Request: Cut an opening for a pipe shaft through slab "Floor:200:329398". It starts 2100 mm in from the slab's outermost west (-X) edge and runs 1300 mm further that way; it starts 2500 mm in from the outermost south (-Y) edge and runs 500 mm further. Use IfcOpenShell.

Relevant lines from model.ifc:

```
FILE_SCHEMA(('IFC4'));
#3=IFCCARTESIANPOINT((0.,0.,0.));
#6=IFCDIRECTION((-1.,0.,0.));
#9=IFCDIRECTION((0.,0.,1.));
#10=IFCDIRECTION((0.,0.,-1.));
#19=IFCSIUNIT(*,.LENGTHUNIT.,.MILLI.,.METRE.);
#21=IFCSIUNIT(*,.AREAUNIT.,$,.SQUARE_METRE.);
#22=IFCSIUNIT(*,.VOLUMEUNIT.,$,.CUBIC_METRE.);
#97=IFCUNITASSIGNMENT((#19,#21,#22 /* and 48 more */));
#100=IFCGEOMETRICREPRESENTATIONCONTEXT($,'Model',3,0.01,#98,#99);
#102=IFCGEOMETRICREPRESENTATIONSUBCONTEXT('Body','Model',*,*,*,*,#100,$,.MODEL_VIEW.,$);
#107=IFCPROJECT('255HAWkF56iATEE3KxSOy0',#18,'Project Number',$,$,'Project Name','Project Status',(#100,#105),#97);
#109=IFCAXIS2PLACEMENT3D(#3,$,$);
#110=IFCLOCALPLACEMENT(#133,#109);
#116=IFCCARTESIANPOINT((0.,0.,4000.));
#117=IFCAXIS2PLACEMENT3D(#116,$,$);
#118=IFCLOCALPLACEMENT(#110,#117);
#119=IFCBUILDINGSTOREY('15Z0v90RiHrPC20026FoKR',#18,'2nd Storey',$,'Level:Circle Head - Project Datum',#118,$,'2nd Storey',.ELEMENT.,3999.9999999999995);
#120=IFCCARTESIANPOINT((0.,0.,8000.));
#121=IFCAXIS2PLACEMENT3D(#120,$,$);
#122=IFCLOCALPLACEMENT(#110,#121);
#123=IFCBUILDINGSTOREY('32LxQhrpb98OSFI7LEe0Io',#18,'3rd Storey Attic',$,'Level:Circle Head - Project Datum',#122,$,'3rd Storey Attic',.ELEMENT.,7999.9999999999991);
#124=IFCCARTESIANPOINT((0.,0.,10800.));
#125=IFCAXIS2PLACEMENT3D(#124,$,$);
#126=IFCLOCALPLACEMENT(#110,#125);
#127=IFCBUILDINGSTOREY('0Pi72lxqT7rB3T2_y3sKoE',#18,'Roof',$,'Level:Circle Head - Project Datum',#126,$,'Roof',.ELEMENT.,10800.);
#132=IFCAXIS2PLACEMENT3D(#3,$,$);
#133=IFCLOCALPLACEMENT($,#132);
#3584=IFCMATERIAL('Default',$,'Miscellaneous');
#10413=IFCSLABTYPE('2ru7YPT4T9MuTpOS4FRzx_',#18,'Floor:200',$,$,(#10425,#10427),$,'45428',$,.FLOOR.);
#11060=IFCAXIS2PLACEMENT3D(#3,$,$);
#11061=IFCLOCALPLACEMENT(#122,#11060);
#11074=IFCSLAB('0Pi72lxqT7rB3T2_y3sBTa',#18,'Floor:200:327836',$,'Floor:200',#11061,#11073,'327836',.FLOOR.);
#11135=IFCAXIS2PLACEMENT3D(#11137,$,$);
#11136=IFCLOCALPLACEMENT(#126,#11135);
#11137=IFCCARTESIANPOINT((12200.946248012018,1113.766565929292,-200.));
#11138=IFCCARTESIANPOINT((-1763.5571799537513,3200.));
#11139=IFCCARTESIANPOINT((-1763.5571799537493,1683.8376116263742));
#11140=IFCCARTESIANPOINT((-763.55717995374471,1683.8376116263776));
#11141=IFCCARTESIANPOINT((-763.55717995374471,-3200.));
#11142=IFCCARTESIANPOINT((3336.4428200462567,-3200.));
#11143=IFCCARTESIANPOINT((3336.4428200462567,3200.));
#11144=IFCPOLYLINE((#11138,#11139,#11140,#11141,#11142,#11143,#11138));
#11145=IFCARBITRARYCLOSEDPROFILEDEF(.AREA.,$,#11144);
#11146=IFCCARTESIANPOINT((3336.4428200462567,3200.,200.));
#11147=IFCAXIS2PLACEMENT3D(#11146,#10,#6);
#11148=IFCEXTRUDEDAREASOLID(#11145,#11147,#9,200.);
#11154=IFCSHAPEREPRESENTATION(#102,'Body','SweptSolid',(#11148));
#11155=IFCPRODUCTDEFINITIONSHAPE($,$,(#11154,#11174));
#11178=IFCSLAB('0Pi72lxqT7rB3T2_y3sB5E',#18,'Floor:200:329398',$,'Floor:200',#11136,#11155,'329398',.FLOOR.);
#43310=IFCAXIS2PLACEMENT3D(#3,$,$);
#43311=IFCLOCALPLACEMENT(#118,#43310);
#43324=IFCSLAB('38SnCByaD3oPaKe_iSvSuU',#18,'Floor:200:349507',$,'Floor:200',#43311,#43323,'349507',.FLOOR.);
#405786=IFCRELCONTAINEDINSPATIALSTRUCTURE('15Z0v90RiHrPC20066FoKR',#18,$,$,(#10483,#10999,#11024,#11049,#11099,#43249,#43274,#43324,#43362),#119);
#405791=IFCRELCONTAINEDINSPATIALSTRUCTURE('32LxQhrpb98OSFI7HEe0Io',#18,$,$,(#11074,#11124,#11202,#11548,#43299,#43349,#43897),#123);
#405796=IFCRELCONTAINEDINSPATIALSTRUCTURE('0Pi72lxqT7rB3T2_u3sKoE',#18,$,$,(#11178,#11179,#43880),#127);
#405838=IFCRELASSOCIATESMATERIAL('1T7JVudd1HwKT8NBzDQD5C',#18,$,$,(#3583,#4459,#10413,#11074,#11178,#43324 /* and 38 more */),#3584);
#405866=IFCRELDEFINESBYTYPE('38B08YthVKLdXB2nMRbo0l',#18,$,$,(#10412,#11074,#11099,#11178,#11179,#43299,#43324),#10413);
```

```python
import numpy as np
import ifcopenshell
import ifcopenshell.api.feature
import ifcopenshell.api.geometry
import ifcopenshell.api.root
import ifcopenshell.geom
import ifcopenshell.util.placement
import ifcopenshell.util.representation
import ifcopenshell.util.shape
import ifcopenshell.util.unit

model = ifcopenshell.open("model.ifc")
unit_scale = ifcopenshell.util.unit.calculate_unit_scale(model)
settings = ifcopenshell.geom.settings()


def volume(element):
    """Net volume in cubic metres, openings subtracted."""
    shape = ifcopenshell.geom.create_shape(settings, element)
    return ifcopenshell.util.shape.get_volume(shape.geometry)


slab = model.by_guid("0Pi72lxqT7rB3T2_y3sB5E")
before = volume(slab)

# Extent in the slab's own axes, in metres. The edges named are its -X and -Y sides.
slab_shape = ifcopenshell.geom.create_shape(settings, slab)
vertices = ifcopenshell.util.shape.get_vertices(slab_shape.geometry)
x_min, y_min, bottom = vertices.min(axis=0)
top = vertices[:, 2].max()

opening = ifcopenshell.api.root.create_entity(model, ifc_class="IfcOpeningElement", name="Pipe shaft opening", predefined_type="OPENING")
context = ifcopenshell.util.representation.get_context(model, "Model", "Body", "MODEL_VIEW")
width, depth = 1.3, 0.5
outline = [(0.0, 0.0), (width, 0.0), (width, depth), (0.0, depth), (0.0, 0.0)]
# Overshoot both faces by 50 mm so the cut is clean.
shape = ifcopenshell.api.geometry.add_slab_representation(
    model, context=context, depth=top - bottom + 0.1, polyline=outline
)
ifcopenshell.api.geometry.assign_representation(model, product=opening, representation=shape)

matrix = ifcopenshell.util.placement.get_local_placement(slab.ObjectPlacement)
matrix[:, 3] = matrix @ np.append(np.array([x_min + 2.1, y_min + 2.5, bottom - 0.05]) / unit_scale, 1.0)
ifcopenshell.api.geometry.edit_object_placement(model, product=opening, matrix=matrix, is_si=False)
ifcopenshell.api.feature.add_feature(model, feature=opening, element=slab)

after = volume(slab)

print(f"slab volume {before:.3f} -> {after:.3f} m3")

model.write("model-out.ifc")
```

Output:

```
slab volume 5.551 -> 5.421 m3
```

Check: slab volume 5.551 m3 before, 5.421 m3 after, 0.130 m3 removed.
